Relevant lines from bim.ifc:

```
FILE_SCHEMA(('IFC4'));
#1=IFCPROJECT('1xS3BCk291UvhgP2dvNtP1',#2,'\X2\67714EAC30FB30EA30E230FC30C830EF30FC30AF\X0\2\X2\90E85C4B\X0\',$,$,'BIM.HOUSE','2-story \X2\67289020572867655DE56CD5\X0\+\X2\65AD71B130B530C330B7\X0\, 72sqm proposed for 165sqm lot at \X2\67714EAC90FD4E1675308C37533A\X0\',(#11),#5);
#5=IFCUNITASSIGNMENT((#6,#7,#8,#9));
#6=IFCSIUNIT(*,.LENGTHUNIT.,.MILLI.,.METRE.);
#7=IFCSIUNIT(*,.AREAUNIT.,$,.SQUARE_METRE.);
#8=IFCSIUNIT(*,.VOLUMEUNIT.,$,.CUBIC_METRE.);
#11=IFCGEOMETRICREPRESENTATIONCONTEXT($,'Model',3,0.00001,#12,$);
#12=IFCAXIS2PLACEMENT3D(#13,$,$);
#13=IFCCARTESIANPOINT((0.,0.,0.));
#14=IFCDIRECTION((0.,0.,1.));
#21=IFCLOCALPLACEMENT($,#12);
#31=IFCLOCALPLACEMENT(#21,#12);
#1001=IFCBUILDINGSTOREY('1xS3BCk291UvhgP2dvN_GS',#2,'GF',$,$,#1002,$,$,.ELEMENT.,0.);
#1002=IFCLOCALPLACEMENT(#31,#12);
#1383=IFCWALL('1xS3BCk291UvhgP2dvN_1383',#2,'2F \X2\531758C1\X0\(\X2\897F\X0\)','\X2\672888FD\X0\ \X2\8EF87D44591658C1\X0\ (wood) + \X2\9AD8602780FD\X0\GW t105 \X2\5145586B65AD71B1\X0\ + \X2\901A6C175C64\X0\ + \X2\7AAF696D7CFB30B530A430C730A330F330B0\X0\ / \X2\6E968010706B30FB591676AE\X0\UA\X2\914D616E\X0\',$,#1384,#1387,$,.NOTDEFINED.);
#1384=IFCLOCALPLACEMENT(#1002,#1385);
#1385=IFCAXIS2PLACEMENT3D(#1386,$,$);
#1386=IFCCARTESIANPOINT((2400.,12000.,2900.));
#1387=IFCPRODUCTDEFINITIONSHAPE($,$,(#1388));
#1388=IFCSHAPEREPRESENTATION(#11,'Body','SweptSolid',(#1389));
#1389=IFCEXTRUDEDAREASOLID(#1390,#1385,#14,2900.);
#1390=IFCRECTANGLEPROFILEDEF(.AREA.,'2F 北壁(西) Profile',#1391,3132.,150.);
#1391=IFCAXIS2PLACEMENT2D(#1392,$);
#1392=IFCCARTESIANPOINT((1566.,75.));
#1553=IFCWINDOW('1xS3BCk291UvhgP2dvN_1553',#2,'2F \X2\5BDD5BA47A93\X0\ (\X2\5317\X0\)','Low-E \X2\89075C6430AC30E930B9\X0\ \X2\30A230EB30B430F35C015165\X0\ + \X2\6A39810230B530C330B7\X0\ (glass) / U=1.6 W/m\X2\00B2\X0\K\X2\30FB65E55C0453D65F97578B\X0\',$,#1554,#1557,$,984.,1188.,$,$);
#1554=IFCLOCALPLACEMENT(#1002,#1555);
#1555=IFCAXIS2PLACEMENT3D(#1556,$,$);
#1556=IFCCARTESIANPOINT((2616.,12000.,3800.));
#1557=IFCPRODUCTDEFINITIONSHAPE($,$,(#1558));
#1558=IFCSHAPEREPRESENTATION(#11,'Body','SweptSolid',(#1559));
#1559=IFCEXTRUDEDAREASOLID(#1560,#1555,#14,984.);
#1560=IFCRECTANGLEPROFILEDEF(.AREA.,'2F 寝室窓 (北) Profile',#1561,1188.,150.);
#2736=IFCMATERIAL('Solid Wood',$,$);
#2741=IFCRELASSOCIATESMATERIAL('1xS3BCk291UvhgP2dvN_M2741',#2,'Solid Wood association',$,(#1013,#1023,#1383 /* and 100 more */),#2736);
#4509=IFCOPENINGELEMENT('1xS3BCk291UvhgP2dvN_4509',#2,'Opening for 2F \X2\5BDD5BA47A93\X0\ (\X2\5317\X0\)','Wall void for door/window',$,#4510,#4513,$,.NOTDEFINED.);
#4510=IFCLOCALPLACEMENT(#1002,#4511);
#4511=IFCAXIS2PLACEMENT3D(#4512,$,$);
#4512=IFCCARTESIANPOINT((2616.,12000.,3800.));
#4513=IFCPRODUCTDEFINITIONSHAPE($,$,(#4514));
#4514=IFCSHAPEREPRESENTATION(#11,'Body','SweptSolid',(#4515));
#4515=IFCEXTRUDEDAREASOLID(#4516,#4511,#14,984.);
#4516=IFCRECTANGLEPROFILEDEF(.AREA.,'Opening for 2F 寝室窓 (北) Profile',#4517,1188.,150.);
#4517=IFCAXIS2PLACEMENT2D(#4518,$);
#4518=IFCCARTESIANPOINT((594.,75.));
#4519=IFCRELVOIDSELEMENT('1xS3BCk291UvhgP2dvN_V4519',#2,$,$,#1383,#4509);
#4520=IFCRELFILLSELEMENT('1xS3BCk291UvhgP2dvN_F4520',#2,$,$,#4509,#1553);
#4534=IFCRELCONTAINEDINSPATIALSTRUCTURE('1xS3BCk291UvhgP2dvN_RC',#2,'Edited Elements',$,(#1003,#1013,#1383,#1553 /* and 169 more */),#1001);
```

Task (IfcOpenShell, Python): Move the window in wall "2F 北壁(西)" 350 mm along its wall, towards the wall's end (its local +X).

```python
import ifcopenshell
import ifcopenshell.api.geometry
import ifcopenshell.util.placement
import ifcopenshell.util.unit

model = ifcopenshell.open("bim.ifc")
unit_scale = ifcopenshell.util.unit.calculate_unit_scale(model)

window = model.by_guid("1xS3BCk291UvhgP2dvN_1553")
opening = window.FillsVoids[0].RelatingOpeningElement
wall = opening.VoidsElements[0].RelatingBuildingElement

wall_matrix = ifcopenshell.util.placement.get_local_placement(wall.ObjectPlacement)
shift = wall_matrix[:3, 0] * 0.35 / unit_scale
before = ifcopenshell.util.placement.get_local_placement(window.ObjectPlacement)[:3, 3].copy()

# The window is not placed relative to its opening, so move both.
for product in (opening, window):
    matrix = ifcopenshell.util.placement.get_local_placement(product.ObjectPlacement)
    matrix[:3, 3] += shift
    ifcopenshell.api.geometry.edit_object_placement(model, product=product, matrix=matrix, is_si=False)

after = ifcopenshell.util.placement.get_local_placement(window.ObjectPlacement)[:3, 3]
print("window moved by", (after - before).round(3) + 0.0)

model.write("bim_updated.ifc")
```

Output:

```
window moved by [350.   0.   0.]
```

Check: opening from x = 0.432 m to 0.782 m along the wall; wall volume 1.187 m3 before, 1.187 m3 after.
